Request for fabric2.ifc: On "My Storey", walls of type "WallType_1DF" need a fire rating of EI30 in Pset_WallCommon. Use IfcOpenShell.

First a look at what the model holds.

```python
import ifcopenshell
import ifcopenshell.util.element

model = ifcopenshell.open("fabric2.ifc")
print(model.schema)
storey = next(s for s in model.by_type("IfcBuildingStorey") if s.Name == "My Storey")
walls = [e for e in ifcopenshell.util.element.get_decomposition(storey) if e.is_a("IfcWall")]
seen = {}
for e in walls:
    element_type = ifcopenshell.util.element.get_type(e)
    key = (element_type.Name if element_type != e and element_type else None, ifcopenshell.util.element.get_pset(e, "Pset_WallCommon", "FireRating"))
    seen[key] = seen.get(key, 0) + 1
for (name, value), count in sorted(seen.items(), key=str):
    print(count, "x", name, "|", value)
```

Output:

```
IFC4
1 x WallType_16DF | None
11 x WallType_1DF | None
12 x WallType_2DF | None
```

```python
import ifcopenshell
import ifcopenshell.api.pset
import ifcopenshell.util.element

model = ifcopenshell.open("fabric2.ifc")

storey = next(s for s in model.by_type("IfcBuildingStorey") if s.Name == "My Storey")
walls = [e for e in ifcopenshell.util.element.get_decomposition(storey) if e.is_a("IfcWall")]

count = 0
for e in walls:
    element_type = ifcopenshell.util.element.get_type(e)
    if element_type in (None, e) or element_type.Name != "WallType_1DF":
        continue
    # add_pset returns the element's existing set when there is one.
    pset = ifcopenshell.api.pset.add_pset(model, product=e, name="Pset_WallCommon")
    ifcopenshell.api.pset.edit_pset(model, pset=pset, properties={"FireRating": "EI30"})
    count += 1

print(count, "walls updated")

model.write("fabric2_edited.ifc")
```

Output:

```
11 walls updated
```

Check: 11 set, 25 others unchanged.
